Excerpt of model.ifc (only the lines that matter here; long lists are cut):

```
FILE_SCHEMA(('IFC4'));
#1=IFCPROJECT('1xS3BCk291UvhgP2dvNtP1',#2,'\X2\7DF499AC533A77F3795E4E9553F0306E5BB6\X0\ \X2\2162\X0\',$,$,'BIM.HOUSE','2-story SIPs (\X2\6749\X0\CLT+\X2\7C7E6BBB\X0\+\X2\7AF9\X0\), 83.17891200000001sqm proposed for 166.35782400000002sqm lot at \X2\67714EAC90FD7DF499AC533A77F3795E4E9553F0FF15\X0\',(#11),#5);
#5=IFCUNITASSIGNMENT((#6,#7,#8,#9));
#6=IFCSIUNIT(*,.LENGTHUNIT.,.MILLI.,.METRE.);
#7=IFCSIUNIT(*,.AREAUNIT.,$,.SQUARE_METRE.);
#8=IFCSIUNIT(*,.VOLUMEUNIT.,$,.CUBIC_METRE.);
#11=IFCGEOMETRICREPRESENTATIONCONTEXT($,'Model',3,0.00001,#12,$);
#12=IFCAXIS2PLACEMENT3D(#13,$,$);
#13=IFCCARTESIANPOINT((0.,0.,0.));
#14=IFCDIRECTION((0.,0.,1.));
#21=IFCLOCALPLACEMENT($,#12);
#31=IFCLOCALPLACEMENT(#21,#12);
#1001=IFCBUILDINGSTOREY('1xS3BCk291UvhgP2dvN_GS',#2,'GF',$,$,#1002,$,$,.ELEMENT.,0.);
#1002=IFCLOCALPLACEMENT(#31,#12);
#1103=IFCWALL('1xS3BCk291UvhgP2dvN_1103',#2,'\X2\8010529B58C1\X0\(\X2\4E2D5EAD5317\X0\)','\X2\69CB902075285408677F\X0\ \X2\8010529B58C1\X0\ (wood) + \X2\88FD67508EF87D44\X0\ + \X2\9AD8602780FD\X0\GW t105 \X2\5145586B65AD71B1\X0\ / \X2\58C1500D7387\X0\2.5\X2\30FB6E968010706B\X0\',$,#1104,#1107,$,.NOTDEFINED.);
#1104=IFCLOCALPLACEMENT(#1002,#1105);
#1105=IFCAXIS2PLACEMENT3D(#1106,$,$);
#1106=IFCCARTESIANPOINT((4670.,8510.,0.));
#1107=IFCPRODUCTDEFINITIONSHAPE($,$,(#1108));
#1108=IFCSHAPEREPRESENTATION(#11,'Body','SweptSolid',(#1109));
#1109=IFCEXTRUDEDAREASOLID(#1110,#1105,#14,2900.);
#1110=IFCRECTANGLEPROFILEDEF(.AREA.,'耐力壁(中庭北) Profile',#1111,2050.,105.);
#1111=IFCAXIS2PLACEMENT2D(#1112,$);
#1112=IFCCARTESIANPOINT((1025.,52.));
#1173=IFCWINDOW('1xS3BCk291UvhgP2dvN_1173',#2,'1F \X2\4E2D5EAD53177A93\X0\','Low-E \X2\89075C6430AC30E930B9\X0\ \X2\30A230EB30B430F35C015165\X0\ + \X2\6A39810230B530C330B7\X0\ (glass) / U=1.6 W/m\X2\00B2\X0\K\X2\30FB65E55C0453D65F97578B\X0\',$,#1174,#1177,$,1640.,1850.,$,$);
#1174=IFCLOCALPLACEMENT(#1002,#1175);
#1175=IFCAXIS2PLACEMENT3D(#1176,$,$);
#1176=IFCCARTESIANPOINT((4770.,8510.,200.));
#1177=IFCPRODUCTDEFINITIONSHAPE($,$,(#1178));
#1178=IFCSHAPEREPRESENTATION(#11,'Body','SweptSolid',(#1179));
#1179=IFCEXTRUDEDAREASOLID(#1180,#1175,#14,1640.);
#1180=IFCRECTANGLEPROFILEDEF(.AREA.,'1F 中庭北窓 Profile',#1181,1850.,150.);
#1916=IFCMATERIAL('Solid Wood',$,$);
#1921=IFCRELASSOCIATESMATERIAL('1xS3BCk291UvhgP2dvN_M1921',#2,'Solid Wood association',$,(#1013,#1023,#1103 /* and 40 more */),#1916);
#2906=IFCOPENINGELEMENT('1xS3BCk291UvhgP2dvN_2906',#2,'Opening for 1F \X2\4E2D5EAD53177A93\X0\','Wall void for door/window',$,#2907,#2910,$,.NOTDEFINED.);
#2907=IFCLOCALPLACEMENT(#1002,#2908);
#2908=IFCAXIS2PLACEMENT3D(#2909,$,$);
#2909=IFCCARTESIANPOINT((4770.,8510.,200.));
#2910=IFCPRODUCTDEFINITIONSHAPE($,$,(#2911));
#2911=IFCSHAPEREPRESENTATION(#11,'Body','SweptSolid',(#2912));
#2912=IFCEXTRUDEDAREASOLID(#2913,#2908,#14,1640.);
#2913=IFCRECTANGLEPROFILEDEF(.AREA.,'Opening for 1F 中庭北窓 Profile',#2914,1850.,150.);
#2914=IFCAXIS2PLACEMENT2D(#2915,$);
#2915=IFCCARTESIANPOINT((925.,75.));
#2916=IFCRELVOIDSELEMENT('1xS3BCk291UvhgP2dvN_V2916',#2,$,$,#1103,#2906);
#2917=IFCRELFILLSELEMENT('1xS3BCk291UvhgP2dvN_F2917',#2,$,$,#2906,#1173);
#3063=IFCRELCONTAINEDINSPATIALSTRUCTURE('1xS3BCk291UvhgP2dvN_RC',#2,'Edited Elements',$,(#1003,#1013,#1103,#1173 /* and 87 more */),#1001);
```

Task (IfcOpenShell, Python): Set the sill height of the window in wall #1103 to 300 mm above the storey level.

```python
import numpy as np
import ifcopenshell
import ifcopenshell.api.geometry
import ifcopenshell.geom
import ifcopenshell.util.element
import ifcopenshell.util.placement
import ifcopenshell.util.shape
import ifcopenshell.util.unit

model = ifcopenshell.open("model.ifc")
unit_scale = ifcopenshell.util.unit.calculate_unit_scale(model)

window = model.by_guid("1xS3BCk291UvhgP2dvN_1173")
opening = window.FillsVoids[0].RelatingOpeningElement
storey = ifcopenshell.util.element.get_container(window, ifc_class="IfcBuildingStorey")
level = ifcopenshell.util.placement.get_local_placement(storey.ObjectPlacement)[2, 3]

# The opening's origin need not be at the sill, so measure its lowest point.
shape = ifcopenshell.geom.create_shape(ifcopenshell.geom.settings(), opening)
bottom = ifcopenshell.util.shape.get_shape_bottom_elevation(shape, shape.geometry) / unit_scale
dz = level + 300.0 - bottom

shift = np.array([0.0, 0.0, dz])
# The window is not placed relative to its opening, so move both.
for product in (opening, window):
    matrix = ifcopenshell.util.placement.get_local_placement(product.ObjectPlacement)
    matrix[:3, 3] += shift
    ifcopenshell.api.geometry.edit_object_placement(model, product=product, matrix=matrix, is_si=False)

print(f"moved by {dz * unit_scale:+.3f} m")

model.write("model_rev.ifc")
```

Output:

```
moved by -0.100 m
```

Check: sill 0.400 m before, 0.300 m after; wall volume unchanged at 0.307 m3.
